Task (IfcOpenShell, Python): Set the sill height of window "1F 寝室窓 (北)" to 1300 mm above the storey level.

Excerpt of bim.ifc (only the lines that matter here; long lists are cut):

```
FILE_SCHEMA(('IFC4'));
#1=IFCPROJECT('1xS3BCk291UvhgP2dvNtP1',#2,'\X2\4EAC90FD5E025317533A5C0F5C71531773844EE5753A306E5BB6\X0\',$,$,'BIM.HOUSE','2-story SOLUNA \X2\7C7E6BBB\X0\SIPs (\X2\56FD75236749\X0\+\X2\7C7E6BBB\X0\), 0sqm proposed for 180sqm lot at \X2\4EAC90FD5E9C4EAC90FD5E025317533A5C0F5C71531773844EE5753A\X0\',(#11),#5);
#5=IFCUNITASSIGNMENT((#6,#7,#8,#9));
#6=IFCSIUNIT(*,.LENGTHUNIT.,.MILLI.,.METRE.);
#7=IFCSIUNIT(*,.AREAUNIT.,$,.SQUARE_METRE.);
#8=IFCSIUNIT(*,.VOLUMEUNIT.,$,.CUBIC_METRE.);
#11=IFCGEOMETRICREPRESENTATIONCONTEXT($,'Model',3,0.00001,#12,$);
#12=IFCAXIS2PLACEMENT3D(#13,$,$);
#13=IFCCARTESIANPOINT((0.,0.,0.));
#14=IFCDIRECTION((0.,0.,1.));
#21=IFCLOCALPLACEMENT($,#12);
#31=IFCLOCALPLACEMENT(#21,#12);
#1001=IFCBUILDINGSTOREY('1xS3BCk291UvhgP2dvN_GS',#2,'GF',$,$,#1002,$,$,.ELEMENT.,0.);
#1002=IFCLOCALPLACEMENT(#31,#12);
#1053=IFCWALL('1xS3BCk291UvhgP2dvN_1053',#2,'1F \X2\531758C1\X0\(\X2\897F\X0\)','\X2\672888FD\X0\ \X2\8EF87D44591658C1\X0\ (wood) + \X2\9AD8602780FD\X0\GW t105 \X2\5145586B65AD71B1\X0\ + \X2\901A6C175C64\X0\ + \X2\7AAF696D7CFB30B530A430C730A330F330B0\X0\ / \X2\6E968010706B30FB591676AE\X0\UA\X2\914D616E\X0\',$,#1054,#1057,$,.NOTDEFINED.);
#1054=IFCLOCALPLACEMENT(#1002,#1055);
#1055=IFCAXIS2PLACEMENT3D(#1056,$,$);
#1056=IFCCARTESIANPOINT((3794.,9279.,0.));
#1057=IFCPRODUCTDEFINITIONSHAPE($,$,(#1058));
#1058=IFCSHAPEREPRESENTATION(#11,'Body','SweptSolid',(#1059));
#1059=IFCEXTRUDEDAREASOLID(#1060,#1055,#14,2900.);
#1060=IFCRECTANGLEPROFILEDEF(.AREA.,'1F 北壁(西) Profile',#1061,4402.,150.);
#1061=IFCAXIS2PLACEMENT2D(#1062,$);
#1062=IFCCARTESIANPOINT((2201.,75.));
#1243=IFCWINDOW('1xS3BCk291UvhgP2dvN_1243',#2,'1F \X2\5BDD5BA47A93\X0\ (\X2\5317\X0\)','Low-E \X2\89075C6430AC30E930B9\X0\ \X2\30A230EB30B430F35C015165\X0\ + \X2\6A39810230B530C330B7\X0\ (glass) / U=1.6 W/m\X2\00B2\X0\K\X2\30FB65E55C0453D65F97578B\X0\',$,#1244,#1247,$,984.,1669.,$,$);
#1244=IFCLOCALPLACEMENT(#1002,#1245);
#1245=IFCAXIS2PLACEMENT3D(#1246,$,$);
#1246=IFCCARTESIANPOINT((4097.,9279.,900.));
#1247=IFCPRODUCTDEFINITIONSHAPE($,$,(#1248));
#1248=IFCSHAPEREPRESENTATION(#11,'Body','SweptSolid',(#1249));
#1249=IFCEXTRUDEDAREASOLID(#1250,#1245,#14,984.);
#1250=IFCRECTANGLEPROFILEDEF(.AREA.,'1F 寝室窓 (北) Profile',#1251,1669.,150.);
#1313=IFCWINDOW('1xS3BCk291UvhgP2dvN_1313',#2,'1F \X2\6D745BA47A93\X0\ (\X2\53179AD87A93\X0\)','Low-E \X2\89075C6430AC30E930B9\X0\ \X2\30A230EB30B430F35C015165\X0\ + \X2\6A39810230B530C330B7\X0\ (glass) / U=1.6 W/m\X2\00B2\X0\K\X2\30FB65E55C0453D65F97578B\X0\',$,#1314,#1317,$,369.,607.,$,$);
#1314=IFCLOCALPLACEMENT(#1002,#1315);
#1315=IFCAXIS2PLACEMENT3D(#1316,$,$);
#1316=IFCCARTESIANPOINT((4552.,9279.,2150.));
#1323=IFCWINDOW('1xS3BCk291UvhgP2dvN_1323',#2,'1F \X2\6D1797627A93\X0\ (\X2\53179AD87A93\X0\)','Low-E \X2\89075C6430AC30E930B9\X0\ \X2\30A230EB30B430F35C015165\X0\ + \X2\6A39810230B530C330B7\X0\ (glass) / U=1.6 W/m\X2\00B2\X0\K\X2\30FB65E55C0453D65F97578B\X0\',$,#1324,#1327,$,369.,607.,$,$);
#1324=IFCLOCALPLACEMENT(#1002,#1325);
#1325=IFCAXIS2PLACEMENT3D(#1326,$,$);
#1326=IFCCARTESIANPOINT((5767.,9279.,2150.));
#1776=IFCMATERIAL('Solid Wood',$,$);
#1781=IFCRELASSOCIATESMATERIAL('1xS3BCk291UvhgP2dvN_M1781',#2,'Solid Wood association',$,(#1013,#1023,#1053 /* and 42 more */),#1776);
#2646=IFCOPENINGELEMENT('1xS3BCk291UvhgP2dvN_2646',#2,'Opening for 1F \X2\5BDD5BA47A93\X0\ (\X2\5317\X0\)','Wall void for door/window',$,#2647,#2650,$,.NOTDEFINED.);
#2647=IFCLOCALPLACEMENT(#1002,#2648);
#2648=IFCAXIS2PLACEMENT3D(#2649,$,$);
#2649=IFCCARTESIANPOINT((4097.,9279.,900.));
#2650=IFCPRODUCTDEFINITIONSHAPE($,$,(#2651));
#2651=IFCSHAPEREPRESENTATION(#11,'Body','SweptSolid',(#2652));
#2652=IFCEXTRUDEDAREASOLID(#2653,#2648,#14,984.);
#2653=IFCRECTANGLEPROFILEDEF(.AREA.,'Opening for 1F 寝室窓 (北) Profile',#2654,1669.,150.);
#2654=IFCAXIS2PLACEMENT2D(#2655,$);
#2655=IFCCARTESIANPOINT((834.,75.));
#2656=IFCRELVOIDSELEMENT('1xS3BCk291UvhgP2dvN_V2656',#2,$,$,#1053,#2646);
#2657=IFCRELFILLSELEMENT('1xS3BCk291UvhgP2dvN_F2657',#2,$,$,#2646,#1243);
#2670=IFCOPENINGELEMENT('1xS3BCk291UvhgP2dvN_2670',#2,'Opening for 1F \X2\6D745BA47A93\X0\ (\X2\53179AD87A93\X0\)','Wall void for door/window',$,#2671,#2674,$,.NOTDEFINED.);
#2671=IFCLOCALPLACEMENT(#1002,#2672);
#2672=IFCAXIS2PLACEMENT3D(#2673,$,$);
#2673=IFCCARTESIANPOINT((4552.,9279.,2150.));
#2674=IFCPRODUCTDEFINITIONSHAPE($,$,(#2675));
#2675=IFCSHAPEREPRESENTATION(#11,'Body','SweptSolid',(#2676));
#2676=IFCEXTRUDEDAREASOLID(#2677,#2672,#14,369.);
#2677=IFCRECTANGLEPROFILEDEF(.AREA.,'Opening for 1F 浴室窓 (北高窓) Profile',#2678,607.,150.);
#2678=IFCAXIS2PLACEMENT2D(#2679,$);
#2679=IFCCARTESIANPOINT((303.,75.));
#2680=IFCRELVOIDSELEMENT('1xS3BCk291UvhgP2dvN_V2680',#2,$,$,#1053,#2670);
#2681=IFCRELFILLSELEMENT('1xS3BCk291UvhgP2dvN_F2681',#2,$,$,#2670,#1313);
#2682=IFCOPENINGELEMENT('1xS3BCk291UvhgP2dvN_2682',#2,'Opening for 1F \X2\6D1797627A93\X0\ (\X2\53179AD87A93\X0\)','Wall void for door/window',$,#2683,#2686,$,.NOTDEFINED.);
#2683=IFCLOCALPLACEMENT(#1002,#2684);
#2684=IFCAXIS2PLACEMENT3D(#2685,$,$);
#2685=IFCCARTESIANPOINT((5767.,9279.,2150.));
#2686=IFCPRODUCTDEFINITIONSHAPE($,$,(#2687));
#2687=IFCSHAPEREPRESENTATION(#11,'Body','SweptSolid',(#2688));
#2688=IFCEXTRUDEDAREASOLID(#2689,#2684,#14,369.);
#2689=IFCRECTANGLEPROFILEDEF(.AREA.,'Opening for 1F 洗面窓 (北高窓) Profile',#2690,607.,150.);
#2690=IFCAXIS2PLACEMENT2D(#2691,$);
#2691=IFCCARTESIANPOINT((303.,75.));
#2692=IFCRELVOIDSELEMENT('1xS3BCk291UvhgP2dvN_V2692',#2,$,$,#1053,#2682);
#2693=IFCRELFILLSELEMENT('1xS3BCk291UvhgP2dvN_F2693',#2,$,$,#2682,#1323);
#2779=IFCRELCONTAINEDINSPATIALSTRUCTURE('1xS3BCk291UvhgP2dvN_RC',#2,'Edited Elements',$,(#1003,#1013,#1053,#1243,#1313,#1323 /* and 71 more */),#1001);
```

```python
import numpy as np
import ifcopenshell
import ifcopenshell.api.geometry
import ifcopenshell.geom
import ifcopenshell.util.element
import ifcopenshell.util.placement
import ifcopenshell.util.shape
import ifcopenshell.util.unit

model = ifcopenshell.open("bim.ifc")
unit_scale = ifcopenshell.util.unit.calculate_unit_scale(model)

window = model.by_id(1243)
opening = window.FillsVoids[0].RelatingOpeningElement
storey = ifcopenshell.util.element.get_container(window, ifc_class="IfcBuildingStorey")
level = ifcopenshell.util.placement.get_local_placement(storey.ObjectPlacement)[2, 3]

# The opening's origin need not be at the sill, so measure its lowest point.
shape = ifcopenshell.geom.create_shape(ifcopenshell.geom.settings(), opening)
bottom = ifcopenshell.util.shape.get_shape_bottom_elevation(shape, shape.geometry) / unit_scale
dz = level + 1.3 / unit_scale - bottom

shift = np.array([0.0, 0.0, dz])
# The window is not placed relative to its opening, so move both.
for product in (opening, window):
    matrix = ifcopenshell.util.placement.get_local_placement(product.ObjectPlacement)
    matrix[:3, 3] += shift
    ifcopenshell.api.geometry.edit_object_placement(model, product=product, matrix=matrix, is_si=False)

print(f"moved by {dz * unit_scale:+.3f} m")

model.write("bim_rev.ifc")
```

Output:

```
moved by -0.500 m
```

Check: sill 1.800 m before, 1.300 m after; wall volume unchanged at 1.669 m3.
